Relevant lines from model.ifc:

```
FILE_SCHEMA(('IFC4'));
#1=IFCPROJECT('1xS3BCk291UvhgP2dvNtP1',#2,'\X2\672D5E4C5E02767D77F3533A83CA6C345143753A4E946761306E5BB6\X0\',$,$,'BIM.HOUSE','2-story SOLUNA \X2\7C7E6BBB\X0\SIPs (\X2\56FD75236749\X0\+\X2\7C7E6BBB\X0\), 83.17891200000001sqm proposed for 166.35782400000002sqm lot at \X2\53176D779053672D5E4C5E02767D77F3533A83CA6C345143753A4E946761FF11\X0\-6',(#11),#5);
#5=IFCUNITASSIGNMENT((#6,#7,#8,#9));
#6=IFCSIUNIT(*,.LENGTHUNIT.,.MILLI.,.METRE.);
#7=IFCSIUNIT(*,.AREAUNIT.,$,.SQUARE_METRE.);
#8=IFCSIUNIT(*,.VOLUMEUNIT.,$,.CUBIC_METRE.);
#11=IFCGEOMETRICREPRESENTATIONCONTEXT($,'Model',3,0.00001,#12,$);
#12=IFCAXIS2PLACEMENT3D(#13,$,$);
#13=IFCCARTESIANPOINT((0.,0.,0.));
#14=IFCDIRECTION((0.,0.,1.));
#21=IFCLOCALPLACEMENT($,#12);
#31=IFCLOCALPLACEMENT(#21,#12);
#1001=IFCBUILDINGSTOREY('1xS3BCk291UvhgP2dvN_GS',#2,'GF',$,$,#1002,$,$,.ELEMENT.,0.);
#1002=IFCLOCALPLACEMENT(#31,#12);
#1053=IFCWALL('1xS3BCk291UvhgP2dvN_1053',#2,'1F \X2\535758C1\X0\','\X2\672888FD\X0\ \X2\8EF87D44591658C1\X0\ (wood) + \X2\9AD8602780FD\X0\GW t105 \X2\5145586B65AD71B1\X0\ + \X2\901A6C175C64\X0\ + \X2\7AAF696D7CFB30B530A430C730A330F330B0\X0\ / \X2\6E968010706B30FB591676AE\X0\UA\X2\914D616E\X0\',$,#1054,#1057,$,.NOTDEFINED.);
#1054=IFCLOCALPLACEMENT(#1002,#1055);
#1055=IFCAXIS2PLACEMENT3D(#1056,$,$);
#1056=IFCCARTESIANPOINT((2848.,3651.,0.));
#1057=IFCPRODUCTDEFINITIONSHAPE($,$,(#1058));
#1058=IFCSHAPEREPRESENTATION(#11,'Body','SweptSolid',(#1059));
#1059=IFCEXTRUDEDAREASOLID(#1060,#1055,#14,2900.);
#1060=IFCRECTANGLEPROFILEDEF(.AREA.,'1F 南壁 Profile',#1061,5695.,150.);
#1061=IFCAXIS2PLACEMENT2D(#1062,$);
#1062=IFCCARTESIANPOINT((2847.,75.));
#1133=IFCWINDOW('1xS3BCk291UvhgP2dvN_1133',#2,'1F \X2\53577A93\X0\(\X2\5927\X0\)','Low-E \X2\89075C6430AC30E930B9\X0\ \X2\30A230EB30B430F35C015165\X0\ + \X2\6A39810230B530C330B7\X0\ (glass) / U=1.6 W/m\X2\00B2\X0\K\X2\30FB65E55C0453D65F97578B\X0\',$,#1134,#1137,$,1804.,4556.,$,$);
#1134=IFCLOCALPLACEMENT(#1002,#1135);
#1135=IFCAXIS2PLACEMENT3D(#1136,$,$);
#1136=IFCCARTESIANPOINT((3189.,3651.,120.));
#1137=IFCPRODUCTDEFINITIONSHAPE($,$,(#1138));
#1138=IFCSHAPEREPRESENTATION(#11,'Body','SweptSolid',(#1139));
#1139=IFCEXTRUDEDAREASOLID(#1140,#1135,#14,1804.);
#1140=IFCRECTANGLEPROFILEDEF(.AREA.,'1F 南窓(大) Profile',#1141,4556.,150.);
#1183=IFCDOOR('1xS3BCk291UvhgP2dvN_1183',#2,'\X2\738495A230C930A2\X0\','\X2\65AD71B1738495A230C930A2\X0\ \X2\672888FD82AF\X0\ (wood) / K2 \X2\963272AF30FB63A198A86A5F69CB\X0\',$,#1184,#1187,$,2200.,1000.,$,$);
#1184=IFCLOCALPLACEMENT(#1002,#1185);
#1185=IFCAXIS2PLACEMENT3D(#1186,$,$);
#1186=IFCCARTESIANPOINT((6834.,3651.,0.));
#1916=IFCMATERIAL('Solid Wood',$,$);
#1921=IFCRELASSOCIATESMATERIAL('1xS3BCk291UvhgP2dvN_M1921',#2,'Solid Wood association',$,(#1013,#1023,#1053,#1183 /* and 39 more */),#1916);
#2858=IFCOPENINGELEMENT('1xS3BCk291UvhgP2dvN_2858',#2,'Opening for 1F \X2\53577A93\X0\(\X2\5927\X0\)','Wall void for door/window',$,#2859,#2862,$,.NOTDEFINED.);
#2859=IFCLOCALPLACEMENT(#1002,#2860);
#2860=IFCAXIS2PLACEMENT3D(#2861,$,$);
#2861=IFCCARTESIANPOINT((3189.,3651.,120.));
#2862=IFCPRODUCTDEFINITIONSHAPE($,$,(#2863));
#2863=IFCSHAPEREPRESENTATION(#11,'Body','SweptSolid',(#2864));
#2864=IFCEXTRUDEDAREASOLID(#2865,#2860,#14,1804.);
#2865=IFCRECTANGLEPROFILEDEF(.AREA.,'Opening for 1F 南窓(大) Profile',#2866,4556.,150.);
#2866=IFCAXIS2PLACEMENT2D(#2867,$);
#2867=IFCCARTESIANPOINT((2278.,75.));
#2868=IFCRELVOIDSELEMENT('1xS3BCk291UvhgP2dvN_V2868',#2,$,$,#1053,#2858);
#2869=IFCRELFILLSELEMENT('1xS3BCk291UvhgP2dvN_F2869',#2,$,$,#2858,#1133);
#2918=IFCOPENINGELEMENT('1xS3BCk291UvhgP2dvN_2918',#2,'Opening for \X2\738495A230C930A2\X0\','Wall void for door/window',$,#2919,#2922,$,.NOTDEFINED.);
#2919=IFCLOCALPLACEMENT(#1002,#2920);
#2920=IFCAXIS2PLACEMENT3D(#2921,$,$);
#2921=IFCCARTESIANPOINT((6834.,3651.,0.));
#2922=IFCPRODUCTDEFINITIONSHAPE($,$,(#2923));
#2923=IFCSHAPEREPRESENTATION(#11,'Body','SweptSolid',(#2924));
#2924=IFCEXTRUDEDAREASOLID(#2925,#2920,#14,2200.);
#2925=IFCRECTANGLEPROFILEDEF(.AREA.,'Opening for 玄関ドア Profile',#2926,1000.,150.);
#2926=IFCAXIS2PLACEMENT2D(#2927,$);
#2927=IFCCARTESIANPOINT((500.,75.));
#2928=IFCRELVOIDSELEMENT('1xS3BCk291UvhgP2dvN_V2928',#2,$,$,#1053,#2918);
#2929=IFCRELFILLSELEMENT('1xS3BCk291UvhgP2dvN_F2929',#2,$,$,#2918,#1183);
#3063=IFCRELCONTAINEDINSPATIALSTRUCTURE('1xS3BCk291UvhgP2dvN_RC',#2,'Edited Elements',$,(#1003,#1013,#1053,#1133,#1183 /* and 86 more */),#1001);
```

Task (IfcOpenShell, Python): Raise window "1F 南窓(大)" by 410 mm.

```python
import numpy as np
import ifcopenshell
import ifcopenshell.api.geometry
import ifcopenshell.util.placement
import ifcopenshell.util.unit

model = ifcopenshell.open("model.ifc")
unit_scale = ifcopenshell.util.unit.calculate_unit_scale(model)

window = model.by_guid("1xS3BCk291UvhgP2dvN_1133")
opening = window.FillsVoids[0].RelatingOpeningElement
dz = 0.41 / unit_scale

shift = np.array([0.0, 0.0, dz])
# The window is not placed relative to its opening, so move both.
for product in (opening, window):
    matrix = ifcopenshell.util.placement.get_local_placement(product.ObjectPlacement)
    matrix[:3, 3] += shift
    ifcopenshell.api.geometry.edit_object_placement(model, product=product, matrix=matrix, is_si=False)

print(f"moved by {dz * unit_scale:+.3f} m")

model.write("model-out.ifc")
```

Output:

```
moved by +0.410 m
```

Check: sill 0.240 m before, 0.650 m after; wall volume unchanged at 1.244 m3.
